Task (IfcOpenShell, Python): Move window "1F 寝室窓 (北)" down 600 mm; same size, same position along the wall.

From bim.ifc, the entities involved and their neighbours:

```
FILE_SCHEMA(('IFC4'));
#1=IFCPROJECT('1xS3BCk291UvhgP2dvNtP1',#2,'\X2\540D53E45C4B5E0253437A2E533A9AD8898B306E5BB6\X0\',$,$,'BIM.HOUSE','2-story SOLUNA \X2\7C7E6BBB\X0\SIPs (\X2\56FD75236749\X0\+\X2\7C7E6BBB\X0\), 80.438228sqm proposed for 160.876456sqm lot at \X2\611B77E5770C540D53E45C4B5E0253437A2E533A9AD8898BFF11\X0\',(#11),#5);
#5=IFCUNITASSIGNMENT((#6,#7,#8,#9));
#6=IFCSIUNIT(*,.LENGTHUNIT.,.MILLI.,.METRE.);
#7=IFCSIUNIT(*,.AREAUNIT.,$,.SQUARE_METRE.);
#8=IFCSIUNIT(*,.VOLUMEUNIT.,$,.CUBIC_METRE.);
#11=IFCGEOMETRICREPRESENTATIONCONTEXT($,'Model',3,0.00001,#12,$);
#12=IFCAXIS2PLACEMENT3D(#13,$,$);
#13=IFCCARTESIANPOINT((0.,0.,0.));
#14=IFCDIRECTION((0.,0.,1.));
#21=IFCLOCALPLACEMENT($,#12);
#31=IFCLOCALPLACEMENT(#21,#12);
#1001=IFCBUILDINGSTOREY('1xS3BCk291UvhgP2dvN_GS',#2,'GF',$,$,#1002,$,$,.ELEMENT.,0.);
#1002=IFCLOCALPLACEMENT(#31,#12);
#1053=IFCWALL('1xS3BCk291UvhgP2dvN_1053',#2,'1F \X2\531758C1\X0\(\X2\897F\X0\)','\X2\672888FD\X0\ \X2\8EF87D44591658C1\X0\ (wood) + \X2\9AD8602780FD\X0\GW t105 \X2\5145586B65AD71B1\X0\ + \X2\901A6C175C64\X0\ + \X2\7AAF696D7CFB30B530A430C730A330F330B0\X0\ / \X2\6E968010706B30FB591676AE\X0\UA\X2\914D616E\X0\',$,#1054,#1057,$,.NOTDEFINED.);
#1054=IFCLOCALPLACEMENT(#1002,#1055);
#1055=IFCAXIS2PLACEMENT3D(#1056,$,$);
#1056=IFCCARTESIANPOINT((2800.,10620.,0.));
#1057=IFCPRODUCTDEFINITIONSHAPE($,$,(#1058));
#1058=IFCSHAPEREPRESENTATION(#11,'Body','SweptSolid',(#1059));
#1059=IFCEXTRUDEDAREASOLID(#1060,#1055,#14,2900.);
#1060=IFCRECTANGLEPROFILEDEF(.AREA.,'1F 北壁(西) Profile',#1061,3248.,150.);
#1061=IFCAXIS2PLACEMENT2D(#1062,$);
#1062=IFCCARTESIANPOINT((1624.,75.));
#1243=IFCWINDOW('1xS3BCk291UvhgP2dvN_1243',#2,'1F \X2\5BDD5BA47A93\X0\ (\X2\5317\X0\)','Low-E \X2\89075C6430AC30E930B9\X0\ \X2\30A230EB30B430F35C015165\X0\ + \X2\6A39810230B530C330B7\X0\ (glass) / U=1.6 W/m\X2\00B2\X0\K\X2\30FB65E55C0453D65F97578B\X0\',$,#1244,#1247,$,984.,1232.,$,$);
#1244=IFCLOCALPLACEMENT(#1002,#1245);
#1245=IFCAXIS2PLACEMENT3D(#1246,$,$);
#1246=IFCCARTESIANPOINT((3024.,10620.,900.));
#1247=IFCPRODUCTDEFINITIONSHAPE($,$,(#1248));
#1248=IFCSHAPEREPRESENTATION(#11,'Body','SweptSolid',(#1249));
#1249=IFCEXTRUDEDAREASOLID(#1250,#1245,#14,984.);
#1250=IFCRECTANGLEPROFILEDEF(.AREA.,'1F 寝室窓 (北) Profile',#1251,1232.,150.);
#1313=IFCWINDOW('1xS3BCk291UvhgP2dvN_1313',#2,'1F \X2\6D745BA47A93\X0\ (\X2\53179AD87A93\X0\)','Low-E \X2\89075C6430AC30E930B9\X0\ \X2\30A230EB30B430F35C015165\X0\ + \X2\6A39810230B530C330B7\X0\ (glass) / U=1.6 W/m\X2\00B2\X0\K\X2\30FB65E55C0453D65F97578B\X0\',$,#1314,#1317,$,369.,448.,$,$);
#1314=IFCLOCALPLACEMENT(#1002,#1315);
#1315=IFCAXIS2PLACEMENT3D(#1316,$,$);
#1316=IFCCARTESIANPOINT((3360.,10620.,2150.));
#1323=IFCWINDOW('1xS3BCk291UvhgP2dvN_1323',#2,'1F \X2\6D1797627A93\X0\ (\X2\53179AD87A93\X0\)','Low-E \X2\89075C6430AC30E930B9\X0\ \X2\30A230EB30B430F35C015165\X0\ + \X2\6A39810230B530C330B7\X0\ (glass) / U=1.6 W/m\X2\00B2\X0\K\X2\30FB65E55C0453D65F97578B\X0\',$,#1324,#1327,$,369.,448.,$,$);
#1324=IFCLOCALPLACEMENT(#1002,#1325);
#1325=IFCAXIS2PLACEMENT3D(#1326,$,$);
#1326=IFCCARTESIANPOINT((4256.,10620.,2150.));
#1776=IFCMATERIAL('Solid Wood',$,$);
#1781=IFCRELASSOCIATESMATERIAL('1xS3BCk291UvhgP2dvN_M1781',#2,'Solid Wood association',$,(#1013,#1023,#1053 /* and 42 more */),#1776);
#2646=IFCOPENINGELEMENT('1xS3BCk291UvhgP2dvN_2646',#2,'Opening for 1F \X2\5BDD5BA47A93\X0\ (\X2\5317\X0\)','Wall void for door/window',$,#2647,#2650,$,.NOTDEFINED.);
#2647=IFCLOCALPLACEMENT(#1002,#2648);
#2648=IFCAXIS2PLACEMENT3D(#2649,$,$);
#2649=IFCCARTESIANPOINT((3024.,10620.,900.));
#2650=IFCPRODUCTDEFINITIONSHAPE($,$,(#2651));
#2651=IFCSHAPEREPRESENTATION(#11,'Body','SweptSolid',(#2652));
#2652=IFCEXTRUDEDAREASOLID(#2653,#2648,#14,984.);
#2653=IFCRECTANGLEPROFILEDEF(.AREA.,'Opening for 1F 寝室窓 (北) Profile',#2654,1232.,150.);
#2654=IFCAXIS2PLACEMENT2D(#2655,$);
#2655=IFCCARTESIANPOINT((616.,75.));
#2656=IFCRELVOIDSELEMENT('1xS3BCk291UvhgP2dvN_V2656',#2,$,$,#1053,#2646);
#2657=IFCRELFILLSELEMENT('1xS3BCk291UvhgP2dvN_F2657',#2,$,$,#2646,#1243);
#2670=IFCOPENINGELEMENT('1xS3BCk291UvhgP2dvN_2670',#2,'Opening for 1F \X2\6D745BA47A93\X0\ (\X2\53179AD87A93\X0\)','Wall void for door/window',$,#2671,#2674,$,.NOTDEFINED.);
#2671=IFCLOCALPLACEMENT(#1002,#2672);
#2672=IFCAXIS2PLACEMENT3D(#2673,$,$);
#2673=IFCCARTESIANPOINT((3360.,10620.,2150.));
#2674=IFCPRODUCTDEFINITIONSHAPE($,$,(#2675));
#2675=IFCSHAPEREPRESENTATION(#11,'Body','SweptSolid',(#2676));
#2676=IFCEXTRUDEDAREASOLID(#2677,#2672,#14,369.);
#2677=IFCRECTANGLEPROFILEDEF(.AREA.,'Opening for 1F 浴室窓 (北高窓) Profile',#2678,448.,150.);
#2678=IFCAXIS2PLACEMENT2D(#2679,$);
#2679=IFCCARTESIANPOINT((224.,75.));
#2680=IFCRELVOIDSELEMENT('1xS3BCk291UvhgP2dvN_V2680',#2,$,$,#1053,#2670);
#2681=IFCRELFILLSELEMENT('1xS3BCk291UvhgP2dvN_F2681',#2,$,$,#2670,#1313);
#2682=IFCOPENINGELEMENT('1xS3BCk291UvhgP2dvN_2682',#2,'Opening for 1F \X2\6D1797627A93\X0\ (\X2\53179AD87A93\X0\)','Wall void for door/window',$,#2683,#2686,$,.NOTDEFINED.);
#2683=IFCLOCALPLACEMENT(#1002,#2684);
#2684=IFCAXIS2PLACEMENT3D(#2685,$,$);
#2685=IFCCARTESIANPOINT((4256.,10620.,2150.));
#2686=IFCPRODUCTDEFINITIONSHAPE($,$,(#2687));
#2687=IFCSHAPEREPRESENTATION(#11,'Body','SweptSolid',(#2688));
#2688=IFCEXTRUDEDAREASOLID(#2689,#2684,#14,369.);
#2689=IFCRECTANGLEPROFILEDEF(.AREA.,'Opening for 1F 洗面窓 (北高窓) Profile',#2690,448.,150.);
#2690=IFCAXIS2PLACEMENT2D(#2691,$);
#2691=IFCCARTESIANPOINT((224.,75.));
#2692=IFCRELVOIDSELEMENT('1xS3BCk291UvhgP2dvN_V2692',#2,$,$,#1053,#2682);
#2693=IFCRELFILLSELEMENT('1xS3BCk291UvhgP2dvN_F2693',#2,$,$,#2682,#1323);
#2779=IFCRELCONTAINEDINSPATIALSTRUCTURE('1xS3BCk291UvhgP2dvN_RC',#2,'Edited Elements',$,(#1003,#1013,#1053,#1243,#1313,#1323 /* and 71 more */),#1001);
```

```python
import numpy as np
import ifcopenshell
import ifcopenshell.api.geometry
import ifcopenshell.util.placement
import ifcopenshell.util.unit

model = ifcopenshell.open("bim.ifc")
unit_scale = ifcopenshell.util.unit.calculate_unit_scale(model)

window = model.by_guid("1xS3BCk291UvhgP2dvN_1243")
opening = window.FillsVoids[0].RelatingOpeningElement
dz = -600.0

shift = np.array([0.0, 0.0, dz])
# The window is not placed relative to its opening, so move both.
for product in (opening, window):
    matrix = ifcopenshell.util.placement.get_local_placement(product.ObjectPlacement)
    matrix[:3, 3] += shift
    ifcopenshell.api.geometry.edit_object_placement(model, product=product, matrix=matrix, is_si=False)

print(f"moved by {dz * unit_scale:+.3f} m")

model.write("bim_v2.ifc")
```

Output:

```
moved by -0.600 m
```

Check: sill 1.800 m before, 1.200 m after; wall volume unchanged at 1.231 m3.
